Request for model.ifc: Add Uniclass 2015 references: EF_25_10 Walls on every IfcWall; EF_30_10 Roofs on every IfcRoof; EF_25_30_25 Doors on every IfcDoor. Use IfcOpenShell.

First a look at what the model holds.

```python
import ifcopenshell

model = ifcopenshell.open("model.ifc")
print(model.schema)
print("classifications:", [c.Name for c in model.by_type("IfcClassification")])
for ifc_class in ("IfcDoor", "IfcRoof", "IfcStair", "IfcWall", "IfcWindow"):
    print(ifc_class, len(model.by_type(ifc_class)))
```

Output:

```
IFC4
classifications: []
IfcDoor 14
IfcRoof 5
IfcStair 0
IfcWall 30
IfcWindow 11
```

```python
import ifcopenshell
import ifcopenshell.api.classification

model = ifcopenshell.open("model.ifc")

system = ifcopenshell.api.classification.add_classification(model, classification="Uniclass 2015")

codes = {
    "IfcWall": ("EF_25_10", "Walls"),
    "IfcRoof": ("EF_30_10", "Roofs"),
    "IfcDoor": ("EF_25_30_25", "Doors"),
}
for ifc_class, (code, name) in codes.items():
    products = model.by_type(ifc_class)
    ifcopenshell.api.classification.add_reference(
        model, products=products, classification=system, identification=code, name=name
    )
    print(code, len(products))

model.write("model_edited.ifc")
```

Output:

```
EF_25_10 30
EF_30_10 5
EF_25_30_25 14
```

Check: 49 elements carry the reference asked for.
